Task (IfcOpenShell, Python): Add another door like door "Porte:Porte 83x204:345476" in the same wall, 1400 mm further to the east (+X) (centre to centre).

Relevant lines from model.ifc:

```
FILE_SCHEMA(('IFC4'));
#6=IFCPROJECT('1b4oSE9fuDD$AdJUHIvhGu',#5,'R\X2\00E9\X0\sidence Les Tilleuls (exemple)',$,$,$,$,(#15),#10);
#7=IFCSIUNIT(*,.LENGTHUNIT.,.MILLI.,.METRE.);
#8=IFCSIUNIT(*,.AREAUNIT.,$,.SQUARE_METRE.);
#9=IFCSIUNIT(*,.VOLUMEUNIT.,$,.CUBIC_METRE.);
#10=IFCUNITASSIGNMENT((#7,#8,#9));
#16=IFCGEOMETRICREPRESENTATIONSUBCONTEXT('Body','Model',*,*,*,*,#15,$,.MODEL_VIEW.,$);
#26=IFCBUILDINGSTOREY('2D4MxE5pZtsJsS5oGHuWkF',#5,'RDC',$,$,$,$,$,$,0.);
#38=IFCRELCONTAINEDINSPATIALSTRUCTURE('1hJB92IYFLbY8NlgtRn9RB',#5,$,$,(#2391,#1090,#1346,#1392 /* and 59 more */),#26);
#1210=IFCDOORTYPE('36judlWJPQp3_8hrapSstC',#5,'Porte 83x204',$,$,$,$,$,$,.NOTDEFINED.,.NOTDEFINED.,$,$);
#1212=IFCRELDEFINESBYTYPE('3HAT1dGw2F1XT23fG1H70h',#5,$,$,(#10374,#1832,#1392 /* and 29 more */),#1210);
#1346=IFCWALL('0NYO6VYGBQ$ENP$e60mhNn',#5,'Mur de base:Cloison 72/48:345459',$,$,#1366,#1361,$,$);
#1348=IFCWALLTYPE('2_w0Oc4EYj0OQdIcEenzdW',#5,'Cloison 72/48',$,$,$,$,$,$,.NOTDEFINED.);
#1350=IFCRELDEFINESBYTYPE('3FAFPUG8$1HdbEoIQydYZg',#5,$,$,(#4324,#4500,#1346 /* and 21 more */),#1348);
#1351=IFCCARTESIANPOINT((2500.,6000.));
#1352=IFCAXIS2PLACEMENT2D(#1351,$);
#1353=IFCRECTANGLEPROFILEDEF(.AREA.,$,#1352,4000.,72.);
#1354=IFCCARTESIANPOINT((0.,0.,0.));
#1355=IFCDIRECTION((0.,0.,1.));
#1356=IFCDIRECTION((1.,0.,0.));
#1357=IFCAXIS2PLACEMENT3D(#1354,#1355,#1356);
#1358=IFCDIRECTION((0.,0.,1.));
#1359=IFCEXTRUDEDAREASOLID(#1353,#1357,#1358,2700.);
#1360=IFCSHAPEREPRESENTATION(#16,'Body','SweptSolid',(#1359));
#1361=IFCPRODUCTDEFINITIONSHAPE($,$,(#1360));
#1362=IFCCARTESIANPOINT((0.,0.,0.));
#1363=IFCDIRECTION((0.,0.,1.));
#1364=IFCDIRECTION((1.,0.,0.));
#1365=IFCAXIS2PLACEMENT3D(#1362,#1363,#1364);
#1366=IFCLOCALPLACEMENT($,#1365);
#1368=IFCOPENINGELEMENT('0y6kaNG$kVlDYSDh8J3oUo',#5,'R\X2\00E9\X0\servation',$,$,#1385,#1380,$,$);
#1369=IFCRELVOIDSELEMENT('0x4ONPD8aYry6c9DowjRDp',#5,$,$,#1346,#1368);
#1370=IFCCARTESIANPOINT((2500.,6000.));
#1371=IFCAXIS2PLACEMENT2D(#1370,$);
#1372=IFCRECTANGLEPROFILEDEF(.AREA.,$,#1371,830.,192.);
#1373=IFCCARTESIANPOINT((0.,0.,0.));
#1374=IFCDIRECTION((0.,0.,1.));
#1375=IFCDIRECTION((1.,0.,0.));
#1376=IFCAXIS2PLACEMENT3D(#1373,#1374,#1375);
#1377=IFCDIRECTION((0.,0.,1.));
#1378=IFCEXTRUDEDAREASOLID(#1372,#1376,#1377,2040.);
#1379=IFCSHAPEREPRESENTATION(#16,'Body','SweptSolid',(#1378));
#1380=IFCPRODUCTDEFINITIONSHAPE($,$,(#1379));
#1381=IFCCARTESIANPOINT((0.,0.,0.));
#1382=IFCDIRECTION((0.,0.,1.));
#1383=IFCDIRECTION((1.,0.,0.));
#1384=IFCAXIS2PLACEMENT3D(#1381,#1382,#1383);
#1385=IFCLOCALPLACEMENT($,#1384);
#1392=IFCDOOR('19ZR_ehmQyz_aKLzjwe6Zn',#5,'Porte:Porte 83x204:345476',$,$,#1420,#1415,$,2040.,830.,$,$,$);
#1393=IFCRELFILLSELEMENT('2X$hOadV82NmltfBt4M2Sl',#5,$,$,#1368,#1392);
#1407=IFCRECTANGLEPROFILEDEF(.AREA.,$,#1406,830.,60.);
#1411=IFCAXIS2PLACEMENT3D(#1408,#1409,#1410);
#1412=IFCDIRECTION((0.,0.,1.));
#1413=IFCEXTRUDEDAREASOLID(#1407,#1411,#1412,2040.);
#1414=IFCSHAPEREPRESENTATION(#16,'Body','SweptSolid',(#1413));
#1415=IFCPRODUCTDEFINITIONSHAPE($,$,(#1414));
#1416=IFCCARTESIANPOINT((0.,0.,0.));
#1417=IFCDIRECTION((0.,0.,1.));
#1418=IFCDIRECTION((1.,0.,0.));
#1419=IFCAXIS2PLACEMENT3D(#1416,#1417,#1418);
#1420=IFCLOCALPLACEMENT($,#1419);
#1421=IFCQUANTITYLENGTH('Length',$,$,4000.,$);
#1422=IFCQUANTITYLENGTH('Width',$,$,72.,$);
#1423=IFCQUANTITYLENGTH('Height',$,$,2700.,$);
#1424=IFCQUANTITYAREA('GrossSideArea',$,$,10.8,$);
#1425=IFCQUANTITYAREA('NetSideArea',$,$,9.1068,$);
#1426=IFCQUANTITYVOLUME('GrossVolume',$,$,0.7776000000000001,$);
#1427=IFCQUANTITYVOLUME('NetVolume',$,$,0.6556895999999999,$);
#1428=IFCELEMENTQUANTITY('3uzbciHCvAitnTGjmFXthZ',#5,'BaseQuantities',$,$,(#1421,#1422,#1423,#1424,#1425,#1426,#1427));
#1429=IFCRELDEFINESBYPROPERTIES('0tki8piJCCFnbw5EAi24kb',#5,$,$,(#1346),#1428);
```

```python
import ifcopenshell
import ifcopenshell.api.feature
import ifcopenshell.api.geometry
import ifcopenshell.api.pset
import ifcopenshell.api.root
import ifcopenshell.geom
import ifcopenshell.util.element
import ifcopenshell.util.placement
import ifcopenshell.util.shape
import ifcopenshell.util.unit

model = ifcopenshell.open("model.ifc")
unit_scale = ifcopenshell.util.unit.calculate_unit_scale(model)
area_scale = ifcopenshell.util.unit.calculate_unit_scale(model, "AREAUNIT")
volume_scale = ifcopenshell.util.unit.calculate_unit_scale(model, "VOLUMEUNIT")
settings = ifcopenshell.geom.settings()


def volume(element):
    """Net volume in cubic metres, openings subtracted."""
    shape = ifcopenshell.geom.create_shape(settings, element)
    return ifcopenshell.util.shape.get_volume(shape.geometry)


def reuse_history(source, copy):
    """copy_class also copies each property set's owner history, people and application; keep the originals."""
    for rel in copy.IsDefinedBy:
        if rel.is_a("IfcRelDefinesByProperties") and (history := rel.RelatingPropertyDefinition.OwnerHistory):
            rel.RelatingPropertyDefinition.OwnerHistory = source.OwnerHistory
            ifcopenshell.util.element.remove_deep2(model, history)


door = model.by_id(1392)
opening = door.FillsVoids[0].RelatingOpeningElement
wall = opening.VoidsElements[0].RelatingBuildingElement
before = volume(wall)
shift = ifcopenshell.util.placement.get_local_placement(wall.ObjectPlacement)[:3, 0] * 1.4 / unit_scale

# copy_class copies the void relationship, type, container and properties, but no geometry.
new_opening = ifcopenshell.api.root.copy_class(model, product=opening)
new_opening.Representation = ifcopenshell.util.element.copy_deep(
    model, opening.Representation, exclude=["IfcGeometricRepresentationContext", "IfcRepresentationMap"]
)
reuse_history(opening, new_opening)
new_door = ifcopenshell.api.root.copy_class(model, product=door)
new_door.Representation = ifcopenshell.util.element.copy_deep(
    model, door.Representation, exclude=["IfcGeometricRepresentationContext", "IfcRepresentationMap"]
)
new_door.Name = "Porte:Porte 83x204"
reuse_history(door, new_door)
ifcopenshell.api.feature.add_filling(model, opening=new_opening, element=new_door)

for old, new in ((opening, new_opening), (door, new_door)):
    matrix = ifcopenshell.util.placement.get_local_placement(old.ObjectPlacement)
    matrix[:3, 3] += shift
    ifcopenshell.api.geometry.edit_object_placement(model, product=new, matrix=matrix, is_si=False)

after = volume(wall)
thickness = 0.072  # wall thickness in metres

# Update the wall's stored quantities.
qto = model.by_id(ifcopenshell.util.element.get_pset(wall, "BaseQuantities", should_inherit=False)["id"])
ifcopenshell.api.pset.edit_qto(model, qto=qto, properties={
    "NetSideArea": after / thickness / area_scale,
    "NetVolume": after / volume_scale,
})

print(f"wall volume {before:.3f} -> {after:.3f} m3")

model.write("model_v2.ifc")
```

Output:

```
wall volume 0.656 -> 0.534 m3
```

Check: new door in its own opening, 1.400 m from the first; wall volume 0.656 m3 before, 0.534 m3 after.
